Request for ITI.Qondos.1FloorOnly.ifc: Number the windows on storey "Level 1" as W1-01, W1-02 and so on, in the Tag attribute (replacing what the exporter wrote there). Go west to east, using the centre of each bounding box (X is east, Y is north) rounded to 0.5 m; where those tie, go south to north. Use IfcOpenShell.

First a look at what the model holds.

```python
import ifcopenshell
import ifcopenshell.util.element
import ifcopenshell.util.placement

model = ifcopenshell.open("ITI.Qondos.1FloorOnly.ifc")
print(model.schema)
storey = next(s for s in model.by_type("IfcBuildingStorey") if s.Name == "Level 1")
windows = [e for e in ifcopenshell.util.element.get_decomposition(storey) if e.is_a("IfcWindow")]
for e in sorted(windows, key=lambda e: e.id()):
    origin = ifcopenshell.util.placement.get_local_placement(e.ObjectPlacement)[:3, 3]
    print(e.id(), e.Tag, e.Name, origin.round(2) + 0.0, sep=" | ")
```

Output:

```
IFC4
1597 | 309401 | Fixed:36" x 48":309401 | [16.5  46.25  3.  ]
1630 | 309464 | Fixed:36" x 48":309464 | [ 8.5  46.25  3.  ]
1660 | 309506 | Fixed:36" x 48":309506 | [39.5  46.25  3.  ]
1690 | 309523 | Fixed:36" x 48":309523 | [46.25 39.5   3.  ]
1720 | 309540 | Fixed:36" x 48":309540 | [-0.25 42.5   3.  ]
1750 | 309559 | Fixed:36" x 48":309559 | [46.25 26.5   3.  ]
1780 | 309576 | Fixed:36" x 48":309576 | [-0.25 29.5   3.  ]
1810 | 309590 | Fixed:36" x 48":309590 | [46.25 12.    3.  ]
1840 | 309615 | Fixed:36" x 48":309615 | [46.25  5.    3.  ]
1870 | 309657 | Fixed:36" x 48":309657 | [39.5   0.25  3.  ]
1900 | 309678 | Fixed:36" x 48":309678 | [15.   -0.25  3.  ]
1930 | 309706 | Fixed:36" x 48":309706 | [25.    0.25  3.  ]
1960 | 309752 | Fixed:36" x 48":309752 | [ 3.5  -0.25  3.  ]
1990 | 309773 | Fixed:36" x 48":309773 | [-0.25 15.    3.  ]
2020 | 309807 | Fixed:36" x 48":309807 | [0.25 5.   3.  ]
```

```python
import ifcopenshell
import ifcopenshell.geom
import ifcopenshell.util.element
import ifcopenshell.util.shape

model = ifcopenshell.open("ITI.Qondos.1FloorOnly.ifc")
settings = ifcopenshell.geom.settings()
settings.set("use-world-coords", True)


def centre(element):
    shape = ifcopenshell.geom.create_shape(settings, element)
    return ifcopenshell.util.shape.get_bbox_centroid(shape.geometry)


storey = next(s for s in model.by_type("IfcBuildingStorey") if s.Name == "Level 1")
windows = [e for e in ifcopenshell.util.element.get_decomposition(storey) if e.is_a("IfcWindow")]

# Insertion points can sit at a corner or the storey origin, so sort by the geometry (in metres).
centres = {e: centre(e) for e in windows}
windows.sort(key=lambda e: (round(centres[e][0] / 0.5), centres[e][1]))

for i, e in enumerate(windows, start=1):
    number = f"W1-{i:02d}"
    e.Tag = number
    print(e.id(), number)

model.write("ITI.Qondos.1FloorOnly_rev.ifc")
```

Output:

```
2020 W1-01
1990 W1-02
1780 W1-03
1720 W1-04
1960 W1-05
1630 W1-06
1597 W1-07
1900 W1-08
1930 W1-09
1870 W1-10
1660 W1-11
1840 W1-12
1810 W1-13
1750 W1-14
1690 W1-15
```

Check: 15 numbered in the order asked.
